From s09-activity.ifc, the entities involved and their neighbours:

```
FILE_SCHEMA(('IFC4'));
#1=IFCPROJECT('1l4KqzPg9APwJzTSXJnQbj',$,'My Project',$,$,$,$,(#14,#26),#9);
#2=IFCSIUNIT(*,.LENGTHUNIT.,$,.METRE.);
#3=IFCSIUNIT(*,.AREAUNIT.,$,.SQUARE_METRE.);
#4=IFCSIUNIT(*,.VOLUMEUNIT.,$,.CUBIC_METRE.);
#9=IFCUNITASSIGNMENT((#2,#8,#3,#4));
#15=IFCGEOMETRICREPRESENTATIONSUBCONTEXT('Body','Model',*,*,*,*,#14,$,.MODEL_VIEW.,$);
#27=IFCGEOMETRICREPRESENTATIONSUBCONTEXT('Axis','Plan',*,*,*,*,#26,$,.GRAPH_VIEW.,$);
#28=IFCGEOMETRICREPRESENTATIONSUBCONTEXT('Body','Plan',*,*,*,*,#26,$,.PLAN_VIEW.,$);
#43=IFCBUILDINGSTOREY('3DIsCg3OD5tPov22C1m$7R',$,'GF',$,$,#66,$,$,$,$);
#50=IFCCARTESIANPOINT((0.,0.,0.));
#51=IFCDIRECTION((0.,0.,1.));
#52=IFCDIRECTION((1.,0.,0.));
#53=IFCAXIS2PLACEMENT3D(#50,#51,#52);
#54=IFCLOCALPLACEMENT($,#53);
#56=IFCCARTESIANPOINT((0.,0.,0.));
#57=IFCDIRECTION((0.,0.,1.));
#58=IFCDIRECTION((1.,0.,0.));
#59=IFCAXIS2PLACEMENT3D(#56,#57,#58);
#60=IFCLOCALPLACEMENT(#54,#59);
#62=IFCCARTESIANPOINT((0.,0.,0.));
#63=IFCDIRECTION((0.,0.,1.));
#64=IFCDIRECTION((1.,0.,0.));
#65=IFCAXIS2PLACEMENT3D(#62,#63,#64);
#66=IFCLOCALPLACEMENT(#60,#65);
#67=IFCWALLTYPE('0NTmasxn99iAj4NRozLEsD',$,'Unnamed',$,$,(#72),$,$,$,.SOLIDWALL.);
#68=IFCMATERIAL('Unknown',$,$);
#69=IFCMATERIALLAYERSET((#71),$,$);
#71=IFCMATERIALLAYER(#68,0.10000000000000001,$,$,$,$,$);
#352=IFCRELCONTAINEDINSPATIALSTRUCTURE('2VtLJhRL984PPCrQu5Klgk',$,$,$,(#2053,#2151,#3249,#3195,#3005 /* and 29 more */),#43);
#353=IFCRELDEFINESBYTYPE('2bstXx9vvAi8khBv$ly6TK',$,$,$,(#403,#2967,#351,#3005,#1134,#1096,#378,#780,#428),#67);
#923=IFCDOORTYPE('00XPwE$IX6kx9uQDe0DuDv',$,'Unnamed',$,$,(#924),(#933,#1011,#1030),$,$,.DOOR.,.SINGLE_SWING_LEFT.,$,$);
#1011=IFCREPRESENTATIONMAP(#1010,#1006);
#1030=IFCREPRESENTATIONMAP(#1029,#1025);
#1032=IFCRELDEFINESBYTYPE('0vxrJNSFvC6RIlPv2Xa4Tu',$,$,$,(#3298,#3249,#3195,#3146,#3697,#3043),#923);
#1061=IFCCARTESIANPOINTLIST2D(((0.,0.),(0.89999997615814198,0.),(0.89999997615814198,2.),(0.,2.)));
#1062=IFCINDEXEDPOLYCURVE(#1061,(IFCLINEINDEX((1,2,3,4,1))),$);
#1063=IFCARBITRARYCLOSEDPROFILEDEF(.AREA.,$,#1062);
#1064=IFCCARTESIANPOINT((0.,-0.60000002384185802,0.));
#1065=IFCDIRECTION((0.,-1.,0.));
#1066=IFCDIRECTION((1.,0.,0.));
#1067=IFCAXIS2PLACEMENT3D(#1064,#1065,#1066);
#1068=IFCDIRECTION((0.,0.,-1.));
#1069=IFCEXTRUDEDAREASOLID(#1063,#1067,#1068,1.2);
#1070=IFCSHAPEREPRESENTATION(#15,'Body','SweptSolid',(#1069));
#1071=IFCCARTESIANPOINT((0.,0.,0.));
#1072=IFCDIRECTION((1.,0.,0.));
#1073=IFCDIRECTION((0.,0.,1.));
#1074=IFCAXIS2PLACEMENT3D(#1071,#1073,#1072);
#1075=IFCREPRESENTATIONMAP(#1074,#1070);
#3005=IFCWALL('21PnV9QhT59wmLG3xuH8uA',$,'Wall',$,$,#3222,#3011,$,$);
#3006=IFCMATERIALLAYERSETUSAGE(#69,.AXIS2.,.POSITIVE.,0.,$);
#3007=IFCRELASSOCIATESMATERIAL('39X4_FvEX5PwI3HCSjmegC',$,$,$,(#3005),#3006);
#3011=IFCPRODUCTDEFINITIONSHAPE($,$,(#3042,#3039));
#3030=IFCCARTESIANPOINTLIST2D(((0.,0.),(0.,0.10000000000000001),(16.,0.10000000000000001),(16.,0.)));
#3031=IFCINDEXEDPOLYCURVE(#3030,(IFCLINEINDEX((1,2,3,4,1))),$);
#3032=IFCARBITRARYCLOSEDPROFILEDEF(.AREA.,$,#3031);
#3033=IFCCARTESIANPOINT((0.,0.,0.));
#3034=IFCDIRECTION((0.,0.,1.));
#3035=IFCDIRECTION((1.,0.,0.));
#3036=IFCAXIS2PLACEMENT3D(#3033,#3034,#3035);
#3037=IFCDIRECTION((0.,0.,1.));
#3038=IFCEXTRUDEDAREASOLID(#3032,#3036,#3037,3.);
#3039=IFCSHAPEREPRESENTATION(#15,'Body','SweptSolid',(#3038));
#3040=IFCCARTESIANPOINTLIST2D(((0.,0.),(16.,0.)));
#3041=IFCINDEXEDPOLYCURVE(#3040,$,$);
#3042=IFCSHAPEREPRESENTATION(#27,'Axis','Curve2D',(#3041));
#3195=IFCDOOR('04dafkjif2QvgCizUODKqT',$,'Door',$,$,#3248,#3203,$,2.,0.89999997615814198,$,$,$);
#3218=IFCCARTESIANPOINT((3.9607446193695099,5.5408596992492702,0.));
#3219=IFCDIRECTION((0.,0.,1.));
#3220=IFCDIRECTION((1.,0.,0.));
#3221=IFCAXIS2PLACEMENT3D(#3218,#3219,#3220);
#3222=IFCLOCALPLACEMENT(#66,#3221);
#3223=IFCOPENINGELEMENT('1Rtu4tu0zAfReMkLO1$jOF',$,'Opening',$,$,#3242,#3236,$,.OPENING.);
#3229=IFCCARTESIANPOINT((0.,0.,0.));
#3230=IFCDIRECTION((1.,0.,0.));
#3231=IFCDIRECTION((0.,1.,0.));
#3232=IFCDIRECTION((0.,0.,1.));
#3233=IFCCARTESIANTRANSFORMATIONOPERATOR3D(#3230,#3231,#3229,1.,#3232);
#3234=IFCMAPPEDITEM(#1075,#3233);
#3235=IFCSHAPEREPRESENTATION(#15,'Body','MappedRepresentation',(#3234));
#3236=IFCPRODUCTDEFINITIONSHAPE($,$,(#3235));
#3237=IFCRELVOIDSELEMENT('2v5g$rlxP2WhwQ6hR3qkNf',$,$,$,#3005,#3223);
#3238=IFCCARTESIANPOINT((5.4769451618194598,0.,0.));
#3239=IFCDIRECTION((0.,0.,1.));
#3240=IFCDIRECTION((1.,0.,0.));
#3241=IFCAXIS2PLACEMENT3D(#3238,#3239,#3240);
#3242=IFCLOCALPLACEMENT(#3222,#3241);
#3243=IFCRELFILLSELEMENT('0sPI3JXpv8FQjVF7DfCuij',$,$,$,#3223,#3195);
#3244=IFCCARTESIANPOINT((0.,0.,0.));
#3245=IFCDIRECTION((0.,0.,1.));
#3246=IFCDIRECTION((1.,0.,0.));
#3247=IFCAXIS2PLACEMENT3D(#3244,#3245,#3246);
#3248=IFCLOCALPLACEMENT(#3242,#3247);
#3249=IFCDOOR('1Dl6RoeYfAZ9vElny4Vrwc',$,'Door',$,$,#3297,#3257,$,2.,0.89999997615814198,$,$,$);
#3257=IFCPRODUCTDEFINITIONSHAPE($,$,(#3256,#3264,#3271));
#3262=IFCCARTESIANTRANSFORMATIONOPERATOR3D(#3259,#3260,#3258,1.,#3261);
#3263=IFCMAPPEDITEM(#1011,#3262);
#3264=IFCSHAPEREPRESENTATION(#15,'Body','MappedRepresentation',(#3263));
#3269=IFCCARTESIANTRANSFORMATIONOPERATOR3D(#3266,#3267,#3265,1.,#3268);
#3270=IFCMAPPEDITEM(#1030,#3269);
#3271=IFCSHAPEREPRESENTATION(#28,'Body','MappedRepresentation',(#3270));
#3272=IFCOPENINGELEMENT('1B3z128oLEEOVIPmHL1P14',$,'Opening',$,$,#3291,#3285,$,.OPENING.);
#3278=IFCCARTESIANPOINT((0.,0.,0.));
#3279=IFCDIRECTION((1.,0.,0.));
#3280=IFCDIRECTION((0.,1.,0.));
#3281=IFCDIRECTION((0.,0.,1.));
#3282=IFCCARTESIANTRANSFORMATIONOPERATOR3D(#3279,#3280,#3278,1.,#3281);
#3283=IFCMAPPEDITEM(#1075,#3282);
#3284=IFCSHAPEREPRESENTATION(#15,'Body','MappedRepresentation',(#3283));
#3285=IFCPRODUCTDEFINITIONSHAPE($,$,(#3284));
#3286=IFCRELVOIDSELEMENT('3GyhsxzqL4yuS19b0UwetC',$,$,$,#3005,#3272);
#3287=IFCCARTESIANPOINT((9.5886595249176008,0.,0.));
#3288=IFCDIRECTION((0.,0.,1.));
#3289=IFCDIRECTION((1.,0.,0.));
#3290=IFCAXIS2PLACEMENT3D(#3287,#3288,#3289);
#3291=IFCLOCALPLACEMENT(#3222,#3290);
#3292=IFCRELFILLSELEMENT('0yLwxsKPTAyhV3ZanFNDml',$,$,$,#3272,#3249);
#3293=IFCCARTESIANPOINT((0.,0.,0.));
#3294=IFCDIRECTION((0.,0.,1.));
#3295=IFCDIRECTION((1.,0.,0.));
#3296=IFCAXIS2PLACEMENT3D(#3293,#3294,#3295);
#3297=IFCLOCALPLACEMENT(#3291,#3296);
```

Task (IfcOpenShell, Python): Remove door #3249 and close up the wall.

```python
import ifcopenshell
import ifcopenshell.api.feature
import ifcopenshell.api.root
import ifcopenshell.geom
import ifcopenshell.util.shape

model = ifcopenshell.open("s09-activity.ifc")
settings = ifcopenshell.geom.settings()


def volume(element):
    """Net volume in cubic metres, openings subtracted."""
    shape = ifcopenshell.geom.create_shape(settings, element)
    return ifcopenshell.util.shape.get_volume(shape.geometry)


door = model.by_id(3249)
opening = door.FillsVoids[0].RelatingOpeningElement
wall = opening.VoidsElements[0].RelatingBuildingElement
before = volume(wall)

ifcopenshell.api.root.remove_product(model, product=door)
ifcopenshell.api.feature.remove_feature(model, feature=opening)

after = volume(wall)

print(f"wall volume {before:.3f} -> {after:.3f} m3")

model.write("s09-activity_v2.ifc")
```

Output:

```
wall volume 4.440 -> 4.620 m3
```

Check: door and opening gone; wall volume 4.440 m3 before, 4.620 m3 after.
